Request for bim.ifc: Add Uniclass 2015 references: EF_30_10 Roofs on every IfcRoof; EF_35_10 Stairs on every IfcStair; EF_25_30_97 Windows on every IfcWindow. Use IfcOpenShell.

First a look at what the model holds.

```python
import ifcopenshell

model = ifcopenshell.open("bim.ifc")
print(model.schema)
print("classifications:", [c.Name for c in model.by_type("IfcClassification")])
for ifc_class in ("IfcDoor", "IfcRoof", "IfcStair", "IfcWall", "IfcWindow"):
    print(ifc_class, len(model.by_type(ifc_class)))
```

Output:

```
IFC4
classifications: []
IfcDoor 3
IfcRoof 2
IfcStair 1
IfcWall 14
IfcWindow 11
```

```python
import ifcopenshell
import ifcopenshell.api.classification

model = ifcopenshell.open("bim.ifc")

system = ifcopenshell.api.classification.add_classification(model, classification="Uniclass 2015")

codes = {
    "IfcRoof": ("EF_30_10", "Roofs"),
    "IfcStair": ("EF_35_10", "Stairs"),
    "IfcWindow": ("EF_25_30_97", "Windows"),
}
for ifc_class, (code, name) in codes.items():
    products = model.by_type(ifc_class)
    ifcopenshell.api.classification.add_reference(
        model, products=products, classification=system, identification=code, name=name
    )
    print(code, len(products))

model.write("bim_rev.ifc")
```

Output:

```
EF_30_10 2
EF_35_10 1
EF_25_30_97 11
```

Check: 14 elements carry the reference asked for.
